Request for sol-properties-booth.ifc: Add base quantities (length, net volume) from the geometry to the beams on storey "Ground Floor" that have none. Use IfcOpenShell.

First a look at what the model holds.

```python
import ifcopenshell
import ifcopenshell.util.element
import ifcopenshell.util.unit

model = ifcopenshell.open("sol-properties-booth.ifc")
print(model.schema)
for unit_type in ("LENGTHUNIT", "AREAUNIT", "VOLUMEUNIT"):
    print(unit_type, ifcopenshell.util.unit.calculate_unit_scale(model, unit_type))
storey = next(s for s in model.by_type("IfcBuildingStorey") if s.Name == "Ground Floor")
beams = [e for e in ifcopenshell.util.element.get_decomposition(storey) if e.is_a("IfcBeam")]
for e in sorted(beams, key=lambda e: e.id()):
    print(e.id(), e.is_a(), e.Name, list(ifcopenshell.util.element.get_psets(e, qtos_only=True)), sep=" | ")
```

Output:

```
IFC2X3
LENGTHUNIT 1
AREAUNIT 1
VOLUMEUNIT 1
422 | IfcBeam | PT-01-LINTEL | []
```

```python
import ifcopenshell
import ifcopenshell.api.pset
import ifcopenshell.geom
import ifcopenshell.util.element
import ifcopenshell.util.shape
import ifcopenshell.util.unit

model = ifcopenshell.open("sol-properties-booth.ifc")
unit_scale = ifcopenshell.util.unit.calculate_unit_scale(model)
volume_scale = ifcopenshell.util.unit.calculate_unit_scale(model, "VOLUMEUNIT")
settings = ifcopenshell.geom.settings()

storey = next(s for s in model.by_type("IfcBuildingStorey") if s.Name == "Ground Floor")
beams = [e for e in ifcopenshell.util.element.get_decomposition(storey) if e.is_a("IfcBeam")]

for e in sorted(beams, key=lambda e: e.id()):
    if ifcopenshell.util.element.get_psets(e, qtos_only=True, should_inherit=False):
        continue
    # Geometry comes back in metres, in the element's own axes.
    shape = ifcopenshell.geom.create_shape(settings, e)
    values = {
        "Length": ifcopenshell.util.shape.get_max_xyz(shape.geometry) / unit_scale,
        "NetVolume": ifcopenshell.util.shape.get_volume(shape.geometry) / volume_scale,
    }
    qto = ifcopenshell.api.pset.add_qto(model, product=e, name="BaseQuantities")
    ifcopenshell.api.pset.edit_qto(model, qto=qto, properties=values)
    print(e.id(), {k: round(v, 3) for k, v in values.items()})

model.write("sol-properties-booth_edited.ifc")
```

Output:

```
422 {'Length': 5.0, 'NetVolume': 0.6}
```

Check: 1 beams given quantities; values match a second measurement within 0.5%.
